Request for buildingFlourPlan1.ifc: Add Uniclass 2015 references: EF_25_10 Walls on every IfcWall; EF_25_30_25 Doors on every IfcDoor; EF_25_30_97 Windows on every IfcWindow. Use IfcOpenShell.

First a look at what the model holds.

```python
import ifcopenshell

model = ifcopenshell.open("buildingFlourPlan1.ifc")
print(model.schema)
print("classifications:", [c.Name for c in model.by_type("IfcClassification")])
for ifc_class in ("IfcDoor", "IfcRoof", "IfcStair", "IfcWall", "IfcWindow"):
    print(ifc_class, len(model.by_type(ifc_class)))
```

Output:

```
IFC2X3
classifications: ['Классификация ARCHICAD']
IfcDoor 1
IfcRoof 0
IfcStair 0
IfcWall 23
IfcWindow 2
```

```python
import ifcopenshell
import ifcopenshell.api.classification

model = ifcopenshell.open("buildingFlourPlan1.ifc")

# IFC2X3 requires Source and Edition and has no link from the project to the system.
system = model.create_entity("IfcClassification", Source="NBS", Edition="2015", Name="Uniclass 2015")

codes = {
    "IfcWall": ("EF_25_10", "Walls"),
    "IfcDoor": ("EF_25_30_25", "Doors"),
    "IfcWindow": ("EF_25_30_97", "Windows"),
}
for ifc_class, (code, name) in codes.items():
    products = model.by_type(ifc_class)
    ifcopenshell.api.classification.add_reference(
        model, products=products, classification=system, identification=code, name=name
    )
    print(code, len(products))

model.write("buildingFlourPlan1-out.ifc")
```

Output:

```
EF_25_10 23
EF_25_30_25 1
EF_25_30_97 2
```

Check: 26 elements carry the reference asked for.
